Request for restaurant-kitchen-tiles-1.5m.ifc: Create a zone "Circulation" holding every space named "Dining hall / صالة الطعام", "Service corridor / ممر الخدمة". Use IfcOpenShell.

First a look at what the model holds.

```python
import ifcopenshell

model = ifcopenshell.open("restaurant-kitchen-tiles-1.5m.ifc")
print(model.schema)
seen = {}
for space in model.by_type("IfcSpace"):
    seen[space.LongName] = seen.get(space.LongName, 0) + 1
for name, count in sorted(seen.items(), key=str):
    print(count, "x", name)
print("zones:", [z.Name for z in model.by_type("IfcZone")][:20])
```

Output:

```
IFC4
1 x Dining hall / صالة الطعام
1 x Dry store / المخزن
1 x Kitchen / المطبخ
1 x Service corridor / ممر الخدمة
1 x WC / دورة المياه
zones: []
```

```python
import ifcopenshell
import ifcopenshell.api.group
import ifcopenshell.api.root

model = ifcopenshell.open("restaurant-kitchen-tiles-1.5m.ifc")

names = {"Dining hall / صالة الطعام", "Service corridor / ممر الخدمة"}
spaces = [s for s in model.by_type("IfcSpace") if s.LongName in names]

zone = ifcopenshell.api.root.create_entity(model, ifc_class="IfcZone", name="Circulation")
ifcopenshell.api.group.assign_group(model, products=spaces, group=zone)
print(len(spaces), "spaces in", zone.Name)

model.write("restaurant-kitchen-tiles-1.5m_edited.ifc")
```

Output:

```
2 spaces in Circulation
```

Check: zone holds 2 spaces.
